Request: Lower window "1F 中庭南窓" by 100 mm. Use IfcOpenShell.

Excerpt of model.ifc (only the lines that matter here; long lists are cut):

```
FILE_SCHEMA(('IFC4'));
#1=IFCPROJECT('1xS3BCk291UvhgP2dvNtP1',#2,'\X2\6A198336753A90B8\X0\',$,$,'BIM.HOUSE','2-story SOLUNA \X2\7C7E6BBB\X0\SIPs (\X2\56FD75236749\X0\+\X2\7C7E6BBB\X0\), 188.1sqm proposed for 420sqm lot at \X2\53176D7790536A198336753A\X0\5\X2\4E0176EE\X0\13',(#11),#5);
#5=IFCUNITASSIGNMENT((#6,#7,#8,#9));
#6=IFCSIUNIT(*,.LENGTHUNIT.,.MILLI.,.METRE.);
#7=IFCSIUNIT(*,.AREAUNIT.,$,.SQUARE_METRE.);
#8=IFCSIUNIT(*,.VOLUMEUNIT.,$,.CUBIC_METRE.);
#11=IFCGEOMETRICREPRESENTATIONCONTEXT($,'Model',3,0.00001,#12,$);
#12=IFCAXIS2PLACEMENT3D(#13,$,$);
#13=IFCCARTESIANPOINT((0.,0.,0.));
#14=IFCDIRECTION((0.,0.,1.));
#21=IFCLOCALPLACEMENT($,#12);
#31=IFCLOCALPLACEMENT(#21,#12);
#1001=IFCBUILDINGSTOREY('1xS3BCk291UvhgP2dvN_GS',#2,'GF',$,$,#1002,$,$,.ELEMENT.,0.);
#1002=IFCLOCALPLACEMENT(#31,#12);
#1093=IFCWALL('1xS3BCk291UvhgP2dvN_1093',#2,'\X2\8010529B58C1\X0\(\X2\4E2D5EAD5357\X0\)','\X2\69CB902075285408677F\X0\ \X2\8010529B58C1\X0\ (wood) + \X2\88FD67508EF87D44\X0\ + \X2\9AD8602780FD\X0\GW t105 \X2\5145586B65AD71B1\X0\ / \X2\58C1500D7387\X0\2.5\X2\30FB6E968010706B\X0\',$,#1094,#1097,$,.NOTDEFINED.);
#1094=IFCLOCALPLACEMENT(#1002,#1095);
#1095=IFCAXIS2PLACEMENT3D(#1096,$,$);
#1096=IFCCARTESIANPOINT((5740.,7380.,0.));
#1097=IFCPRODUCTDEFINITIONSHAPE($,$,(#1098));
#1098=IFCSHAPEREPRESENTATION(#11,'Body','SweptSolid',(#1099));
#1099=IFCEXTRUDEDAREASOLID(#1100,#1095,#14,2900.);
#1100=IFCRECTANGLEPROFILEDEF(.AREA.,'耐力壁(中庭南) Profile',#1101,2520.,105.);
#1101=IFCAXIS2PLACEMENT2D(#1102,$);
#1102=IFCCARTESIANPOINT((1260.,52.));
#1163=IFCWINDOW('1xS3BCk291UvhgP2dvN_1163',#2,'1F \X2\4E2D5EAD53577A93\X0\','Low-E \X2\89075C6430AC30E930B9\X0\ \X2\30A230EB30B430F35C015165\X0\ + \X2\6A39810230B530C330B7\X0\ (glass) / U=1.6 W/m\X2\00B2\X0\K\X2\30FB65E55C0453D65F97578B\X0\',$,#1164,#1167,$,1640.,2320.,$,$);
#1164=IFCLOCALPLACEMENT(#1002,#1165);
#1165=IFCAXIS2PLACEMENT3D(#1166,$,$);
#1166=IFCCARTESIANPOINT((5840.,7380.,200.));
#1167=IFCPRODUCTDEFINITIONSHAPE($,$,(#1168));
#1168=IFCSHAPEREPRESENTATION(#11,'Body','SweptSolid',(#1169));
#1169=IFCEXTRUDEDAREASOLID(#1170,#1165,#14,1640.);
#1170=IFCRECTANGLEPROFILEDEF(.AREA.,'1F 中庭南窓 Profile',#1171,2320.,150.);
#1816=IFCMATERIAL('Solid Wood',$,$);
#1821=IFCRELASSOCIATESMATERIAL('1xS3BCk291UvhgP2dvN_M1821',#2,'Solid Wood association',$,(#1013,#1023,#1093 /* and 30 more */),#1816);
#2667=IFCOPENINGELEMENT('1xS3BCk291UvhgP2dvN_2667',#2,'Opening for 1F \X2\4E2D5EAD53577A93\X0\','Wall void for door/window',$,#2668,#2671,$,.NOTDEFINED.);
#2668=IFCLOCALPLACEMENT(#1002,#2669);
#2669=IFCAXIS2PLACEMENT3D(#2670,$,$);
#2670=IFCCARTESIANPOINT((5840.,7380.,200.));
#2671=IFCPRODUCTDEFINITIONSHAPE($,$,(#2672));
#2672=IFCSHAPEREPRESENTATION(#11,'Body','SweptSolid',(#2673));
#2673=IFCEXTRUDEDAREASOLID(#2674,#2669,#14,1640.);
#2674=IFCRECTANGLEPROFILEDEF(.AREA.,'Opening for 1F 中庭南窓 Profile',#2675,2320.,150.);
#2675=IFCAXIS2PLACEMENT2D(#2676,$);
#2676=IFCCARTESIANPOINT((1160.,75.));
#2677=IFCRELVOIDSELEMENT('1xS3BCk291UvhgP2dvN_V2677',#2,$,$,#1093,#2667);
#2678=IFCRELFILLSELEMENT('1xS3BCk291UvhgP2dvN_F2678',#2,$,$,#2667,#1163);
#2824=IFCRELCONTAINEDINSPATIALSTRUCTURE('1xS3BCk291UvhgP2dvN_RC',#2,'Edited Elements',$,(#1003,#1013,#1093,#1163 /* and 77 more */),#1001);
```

```python
import numpy as np
import ifcopenshell
import ifcopenshell.api.geometry
import ifcopenshell.util.placement
import ifcopenshell.util.unit

model = ifcopenshell.open("model.ifc")
unit_scale = ifcopenshell.util.unit.calculate_unit_scale(model)

window = model.by_guid("1xS3BCk291UvhgP2dvN_1163")
opening = window.FillsVoids[0].RelatingOpeningElement
dz = -100.0

shift = np.array([0.0, 0.0, dz])
# The window is not placed relative to its opening, so move both.
for product in (opening, window):
    matrix = ifcopenshell.util.placement.get_local_placement(product.ObjectPlacement)
    matrix[:3, 3] += shift
    ifcopenshell.api.geometry.edit_object_placement(model, product=product, matrix=matrix, is_si=False)

print(f"moved by {dz * unit_scale:+.3f} m")

model.write("model-out.ifc")
```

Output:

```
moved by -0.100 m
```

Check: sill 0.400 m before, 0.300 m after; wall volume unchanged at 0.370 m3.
